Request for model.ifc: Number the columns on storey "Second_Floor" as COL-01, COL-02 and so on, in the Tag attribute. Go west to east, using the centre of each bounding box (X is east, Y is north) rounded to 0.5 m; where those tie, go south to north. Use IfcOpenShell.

First a look at what the model holds.

```python
import ifcopenshell
import ifcopenshell.util.element
import ifcopenshell.util.placement

model = ifcopenshell.open("model.ifc")
print(model.schema)
storey = next(s for s in model.by_type("IfcBuildingStorey") if s.Name == "Second_Floor")
columns = [e for e in ifcopenshell.util.element.get_decomposition(storey) if e.is_a("IfcColumn")]
for e in sorted(columns, key=lambda e: e.id()):
    origin = ifcopenshell.util.placement.get_local_placement(e.ObjectPlacement)[:3, 3]
    print(e.id(), e.Tag, e.Name, origin.round(2) + 0.0, sep=" | ")
```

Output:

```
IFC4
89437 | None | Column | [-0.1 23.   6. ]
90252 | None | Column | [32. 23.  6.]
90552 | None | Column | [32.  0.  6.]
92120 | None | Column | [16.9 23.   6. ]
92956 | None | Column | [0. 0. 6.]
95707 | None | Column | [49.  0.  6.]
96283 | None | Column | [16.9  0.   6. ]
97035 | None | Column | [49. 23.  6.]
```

```python
import ifcopenshell
import ifcopenshell.geom
import ifcopenshell.util.element
import ifcopenshell.util.shape

model = ifcopenshell.open("model.ifc")
settings = ifcopenshell.geom.settings()
settings.set("use-world-coords", True)


def centre(element):
    shape = ifcopenshell.geom.create_shape(settings, element)
    return ifcopenshell.util.shape.get_bbox_centroid(shape.geometry)


storey = next(s for s in model.by_type("IfcBuildingStorey") if s.Name == "Second_Floor")
columns = [e for e in ifcopenshell.util.element.get_decomposition(storey) if e.is_a("IfcColumn")]

# Insertion points can sit at a corner or the storey origin, so sort by the geometry (in metres).
centres = {e: centre(e) for e in columns}
columns.sort(key=lambda e: (round(centres[e][0] / 0.5), centres[e][1]))

for i, e in enumerate(columns, start=1):
    number = f"COL-{i:02d}"
    e.Tag = number
    print(e.id(), number)

model.write("model_edited.ifc")
```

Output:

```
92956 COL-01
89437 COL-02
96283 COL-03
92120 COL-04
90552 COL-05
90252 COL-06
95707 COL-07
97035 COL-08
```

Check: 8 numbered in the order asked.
